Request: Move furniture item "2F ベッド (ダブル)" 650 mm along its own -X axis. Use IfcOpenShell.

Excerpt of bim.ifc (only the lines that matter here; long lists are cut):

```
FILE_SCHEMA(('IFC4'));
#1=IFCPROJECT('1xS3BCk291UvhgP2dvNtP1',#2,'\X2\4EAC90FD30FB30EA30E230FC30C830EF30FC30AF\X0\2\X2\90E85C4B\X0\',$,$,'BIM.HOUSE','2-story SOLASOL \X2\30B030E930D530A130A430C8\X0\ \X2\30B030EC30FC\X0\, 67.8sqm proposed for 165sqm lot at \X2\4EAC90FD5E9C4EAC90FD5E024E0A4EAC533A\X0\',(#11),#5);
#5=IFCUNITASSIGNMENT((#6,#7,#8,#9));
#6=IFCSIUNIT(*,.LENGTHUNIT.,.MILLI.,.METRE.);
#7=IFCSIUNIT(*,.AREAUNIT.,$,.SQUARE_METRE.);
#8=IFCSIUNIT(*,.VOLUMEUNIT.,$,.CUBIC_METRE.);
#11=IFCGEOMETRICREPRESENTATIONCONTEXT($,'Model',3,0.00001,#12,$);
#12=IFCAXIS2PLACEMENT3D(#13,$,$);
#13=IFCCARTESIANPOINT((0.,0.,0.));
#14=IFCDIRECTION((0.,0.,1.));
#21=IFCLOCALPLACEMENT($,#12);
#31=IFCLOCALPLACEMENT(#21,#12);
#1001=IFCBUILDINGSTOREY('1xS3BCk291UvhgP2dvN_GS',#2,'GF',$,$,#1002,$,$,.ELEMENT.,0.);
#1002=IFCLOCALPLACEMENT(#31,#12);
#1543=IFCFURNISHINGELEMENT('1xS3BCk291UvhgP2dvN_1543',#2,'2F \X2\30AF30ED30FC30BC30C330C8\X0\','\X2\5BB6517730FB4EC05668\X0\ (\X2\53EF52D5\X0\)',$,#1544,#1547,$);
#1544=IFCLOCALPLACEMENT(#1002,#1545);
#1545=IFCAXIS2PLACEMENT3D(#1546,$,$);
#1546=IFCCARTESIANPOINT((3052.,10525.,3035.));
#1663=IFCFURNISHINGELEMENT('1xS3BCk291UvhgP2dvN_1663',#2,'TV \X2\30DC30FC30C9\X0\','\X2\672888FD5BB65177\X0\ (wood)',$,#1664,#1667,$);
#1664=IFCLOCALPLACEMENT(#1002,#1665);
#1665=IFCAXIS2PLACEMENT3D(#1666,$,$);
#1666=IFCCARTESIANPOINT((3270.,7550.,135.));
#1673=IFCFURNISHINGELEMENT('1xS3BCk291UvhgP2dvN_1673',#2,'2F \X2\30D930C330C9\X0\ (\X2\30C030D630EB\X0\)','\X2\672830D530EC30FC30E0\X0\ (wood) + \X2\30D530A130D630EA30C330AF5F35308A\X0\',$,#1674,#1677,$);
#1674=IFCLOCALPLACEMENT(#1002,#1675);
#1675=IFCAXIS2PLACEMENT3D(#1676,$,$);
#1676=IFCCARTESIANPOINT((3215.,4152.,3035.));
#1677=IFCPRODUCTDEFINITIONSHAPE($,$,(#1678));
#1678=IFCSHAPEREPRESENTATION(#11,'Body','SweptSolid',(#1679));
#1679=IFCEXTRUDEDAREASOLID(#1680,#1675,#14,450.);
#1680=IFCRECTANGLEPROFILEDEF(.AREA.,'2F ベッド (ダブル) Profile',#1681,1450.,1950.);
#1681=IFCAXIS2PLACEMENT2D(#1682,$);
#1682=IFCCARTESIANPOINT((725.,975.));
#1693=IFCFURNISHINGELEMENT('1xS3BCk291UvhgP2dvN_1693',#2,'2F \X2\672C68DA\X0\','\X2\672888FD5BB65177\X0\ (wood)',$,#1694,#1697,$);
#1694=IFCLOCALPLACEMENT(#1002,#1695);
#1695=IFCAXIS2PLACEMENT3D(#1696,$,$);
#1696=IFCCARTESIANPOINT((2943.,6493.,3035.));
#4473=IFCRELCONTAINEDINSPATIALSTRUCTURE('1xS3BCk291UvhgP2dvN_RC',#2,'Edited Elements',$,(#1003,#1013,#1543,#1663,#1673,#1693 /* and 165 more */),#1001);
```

```python
import ifcopenshell
import ifcopenshell.api.geometry
import ifcopenshell.util.placement

model = ifcopenshell.open("bim.ifc")

item = model.by_guid("1xS3BCk291UvhgP2dvN_1673")
matrix = ifcopenshell.util.placement.get_local_placement(item.ObjectPlacement)
matrix[:3, 3] -= matrix[:3, 0] * 650.0
ifcopenshell.api.geometry.edit_object_placement(model, product=item, matrix=matrix, is_si=False)

print(ifcopenshell.util.placement.get_local_placement(item.ObjectPlacement).round(3) + 0.0)

model.write("bim-out.ifc")
```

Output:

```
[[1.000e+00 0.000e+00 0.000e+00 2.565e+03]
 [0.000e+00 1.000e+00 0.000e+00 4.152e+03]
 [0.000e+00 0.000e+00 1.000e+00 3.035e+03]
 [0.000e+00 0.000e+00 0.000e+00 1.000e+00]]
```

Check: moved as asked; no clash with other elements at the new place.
